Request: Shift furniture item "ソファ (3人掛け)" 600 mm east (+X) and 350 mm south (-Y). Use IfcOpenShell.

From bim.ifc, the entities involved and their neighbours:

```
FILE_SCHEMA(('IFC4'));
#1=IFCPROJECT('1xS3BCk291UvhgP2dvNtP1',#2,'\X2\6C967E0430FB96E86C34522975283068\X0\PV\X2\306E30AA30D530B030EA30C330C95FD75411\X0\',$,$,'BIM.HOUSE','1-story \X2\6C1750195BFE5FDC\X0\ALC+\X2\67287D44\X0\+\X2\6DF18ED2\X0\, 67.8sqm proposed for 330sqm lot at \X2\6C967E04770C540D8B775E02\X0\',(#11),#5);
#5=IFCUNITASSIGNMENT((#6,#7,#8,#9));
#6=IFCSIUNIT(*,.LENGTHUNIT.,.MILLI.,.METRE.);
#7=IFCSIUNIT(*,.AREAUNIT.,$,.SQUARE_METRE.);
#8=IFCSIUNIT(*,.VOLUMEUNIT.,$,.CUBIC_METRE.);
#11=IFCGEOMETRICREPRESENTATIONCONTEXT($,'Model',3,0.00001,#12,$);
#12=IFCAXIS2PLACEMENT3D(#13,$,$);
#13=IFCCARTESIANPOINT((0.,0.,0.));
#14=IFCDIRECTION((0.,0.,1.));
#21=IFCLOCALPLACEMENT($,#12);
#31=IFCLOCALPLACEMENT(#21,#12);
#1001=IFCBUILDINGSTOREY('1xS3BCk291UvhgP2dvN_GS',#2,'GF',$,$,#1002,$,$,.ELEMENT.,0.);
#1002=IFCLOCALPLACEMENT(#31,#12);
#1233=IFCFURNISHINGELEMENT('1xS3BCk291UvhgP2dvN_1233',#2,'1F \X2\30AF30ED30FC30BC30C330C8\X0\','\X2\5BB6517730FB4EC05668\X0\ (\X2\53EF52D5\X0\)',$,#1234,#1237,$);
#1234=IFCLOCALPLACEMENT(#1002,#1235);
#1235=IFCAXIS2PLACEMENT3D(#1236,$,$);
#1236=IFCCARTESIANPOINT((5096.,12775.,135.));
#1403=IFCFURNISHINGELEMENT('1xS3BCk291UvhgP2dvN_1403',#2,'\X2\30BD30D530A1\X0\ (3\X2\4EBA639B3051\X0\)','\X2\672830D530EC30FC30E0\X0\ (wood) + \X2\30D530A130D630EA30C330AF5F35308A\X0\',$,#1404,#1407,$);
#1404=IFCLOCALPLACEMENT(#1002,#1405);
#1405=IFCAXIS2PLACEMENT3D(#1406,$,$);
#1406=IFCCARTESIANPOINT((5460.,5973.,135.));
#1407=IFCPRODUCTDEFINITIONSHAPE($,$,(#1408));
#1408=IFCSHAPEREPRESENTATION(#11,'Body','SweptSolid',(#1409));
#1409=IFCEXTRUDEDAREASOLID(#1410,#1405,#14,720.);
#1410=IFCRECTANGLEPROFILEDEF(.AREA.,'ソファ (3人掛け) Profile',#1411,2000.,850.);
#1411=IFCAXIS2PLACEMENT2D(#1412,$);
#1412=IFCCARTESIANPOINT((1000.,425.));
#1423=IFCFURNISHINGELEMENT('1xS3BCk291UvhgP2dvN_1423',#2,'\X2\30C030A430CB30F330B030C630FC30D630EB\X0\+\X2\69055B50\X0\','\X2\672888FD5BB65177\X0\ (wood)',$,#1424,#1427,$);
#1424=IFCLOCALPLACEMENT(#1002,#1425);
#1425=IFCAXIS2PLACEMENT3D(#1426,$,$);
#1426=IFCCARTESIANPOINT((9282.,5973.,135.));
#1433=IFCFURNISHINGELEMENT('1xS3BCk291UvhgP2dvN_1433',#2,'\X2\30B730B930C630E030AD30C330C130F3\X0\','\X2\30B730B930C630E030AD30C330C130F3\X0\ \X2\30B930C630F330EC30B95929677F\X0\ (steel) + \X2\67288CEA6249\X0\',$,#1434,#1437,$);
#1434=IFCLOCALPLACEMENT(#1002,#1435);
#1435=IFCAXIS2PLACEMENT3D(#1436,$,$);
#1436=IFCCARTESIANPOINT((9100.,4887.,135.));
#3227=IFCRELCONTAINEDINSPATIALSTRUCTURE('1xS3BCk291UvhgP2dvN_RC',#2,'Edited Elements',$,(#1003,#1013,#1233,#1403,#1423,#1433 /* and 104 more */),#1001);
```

```python
import ifcopenshell
import ifcopenshell.api.geometry
import ifcopenshell.util.placement

model = ifcopenshell.open("bim.ifc")

item = model.by_guid("1xS3BCk291UvhgP2dvN_1403")
matrix = ifcopenshell.util.placement.get_local_placement(item.ObjectPlacement)
matrix[0, 3] += 600.0
matrix[1, 3] -= 350.0
ifcopenshell.api.geometry.edit_object_placement(model, product=item, matrix=matrix, is_si=False)

print(ifcopenshell.util.placement.get_local_placement(item.ObjectPlacement).round(3) + 0.0)

model.write("bim_v2.ifc")
```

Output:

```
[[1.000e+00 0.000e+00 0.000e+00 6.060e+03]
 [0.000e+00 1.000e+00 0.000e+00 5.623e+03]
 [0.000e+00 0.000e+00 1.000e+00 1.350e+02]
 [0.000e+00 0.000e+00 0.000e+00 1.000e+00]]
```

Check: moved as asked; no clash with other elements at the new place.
